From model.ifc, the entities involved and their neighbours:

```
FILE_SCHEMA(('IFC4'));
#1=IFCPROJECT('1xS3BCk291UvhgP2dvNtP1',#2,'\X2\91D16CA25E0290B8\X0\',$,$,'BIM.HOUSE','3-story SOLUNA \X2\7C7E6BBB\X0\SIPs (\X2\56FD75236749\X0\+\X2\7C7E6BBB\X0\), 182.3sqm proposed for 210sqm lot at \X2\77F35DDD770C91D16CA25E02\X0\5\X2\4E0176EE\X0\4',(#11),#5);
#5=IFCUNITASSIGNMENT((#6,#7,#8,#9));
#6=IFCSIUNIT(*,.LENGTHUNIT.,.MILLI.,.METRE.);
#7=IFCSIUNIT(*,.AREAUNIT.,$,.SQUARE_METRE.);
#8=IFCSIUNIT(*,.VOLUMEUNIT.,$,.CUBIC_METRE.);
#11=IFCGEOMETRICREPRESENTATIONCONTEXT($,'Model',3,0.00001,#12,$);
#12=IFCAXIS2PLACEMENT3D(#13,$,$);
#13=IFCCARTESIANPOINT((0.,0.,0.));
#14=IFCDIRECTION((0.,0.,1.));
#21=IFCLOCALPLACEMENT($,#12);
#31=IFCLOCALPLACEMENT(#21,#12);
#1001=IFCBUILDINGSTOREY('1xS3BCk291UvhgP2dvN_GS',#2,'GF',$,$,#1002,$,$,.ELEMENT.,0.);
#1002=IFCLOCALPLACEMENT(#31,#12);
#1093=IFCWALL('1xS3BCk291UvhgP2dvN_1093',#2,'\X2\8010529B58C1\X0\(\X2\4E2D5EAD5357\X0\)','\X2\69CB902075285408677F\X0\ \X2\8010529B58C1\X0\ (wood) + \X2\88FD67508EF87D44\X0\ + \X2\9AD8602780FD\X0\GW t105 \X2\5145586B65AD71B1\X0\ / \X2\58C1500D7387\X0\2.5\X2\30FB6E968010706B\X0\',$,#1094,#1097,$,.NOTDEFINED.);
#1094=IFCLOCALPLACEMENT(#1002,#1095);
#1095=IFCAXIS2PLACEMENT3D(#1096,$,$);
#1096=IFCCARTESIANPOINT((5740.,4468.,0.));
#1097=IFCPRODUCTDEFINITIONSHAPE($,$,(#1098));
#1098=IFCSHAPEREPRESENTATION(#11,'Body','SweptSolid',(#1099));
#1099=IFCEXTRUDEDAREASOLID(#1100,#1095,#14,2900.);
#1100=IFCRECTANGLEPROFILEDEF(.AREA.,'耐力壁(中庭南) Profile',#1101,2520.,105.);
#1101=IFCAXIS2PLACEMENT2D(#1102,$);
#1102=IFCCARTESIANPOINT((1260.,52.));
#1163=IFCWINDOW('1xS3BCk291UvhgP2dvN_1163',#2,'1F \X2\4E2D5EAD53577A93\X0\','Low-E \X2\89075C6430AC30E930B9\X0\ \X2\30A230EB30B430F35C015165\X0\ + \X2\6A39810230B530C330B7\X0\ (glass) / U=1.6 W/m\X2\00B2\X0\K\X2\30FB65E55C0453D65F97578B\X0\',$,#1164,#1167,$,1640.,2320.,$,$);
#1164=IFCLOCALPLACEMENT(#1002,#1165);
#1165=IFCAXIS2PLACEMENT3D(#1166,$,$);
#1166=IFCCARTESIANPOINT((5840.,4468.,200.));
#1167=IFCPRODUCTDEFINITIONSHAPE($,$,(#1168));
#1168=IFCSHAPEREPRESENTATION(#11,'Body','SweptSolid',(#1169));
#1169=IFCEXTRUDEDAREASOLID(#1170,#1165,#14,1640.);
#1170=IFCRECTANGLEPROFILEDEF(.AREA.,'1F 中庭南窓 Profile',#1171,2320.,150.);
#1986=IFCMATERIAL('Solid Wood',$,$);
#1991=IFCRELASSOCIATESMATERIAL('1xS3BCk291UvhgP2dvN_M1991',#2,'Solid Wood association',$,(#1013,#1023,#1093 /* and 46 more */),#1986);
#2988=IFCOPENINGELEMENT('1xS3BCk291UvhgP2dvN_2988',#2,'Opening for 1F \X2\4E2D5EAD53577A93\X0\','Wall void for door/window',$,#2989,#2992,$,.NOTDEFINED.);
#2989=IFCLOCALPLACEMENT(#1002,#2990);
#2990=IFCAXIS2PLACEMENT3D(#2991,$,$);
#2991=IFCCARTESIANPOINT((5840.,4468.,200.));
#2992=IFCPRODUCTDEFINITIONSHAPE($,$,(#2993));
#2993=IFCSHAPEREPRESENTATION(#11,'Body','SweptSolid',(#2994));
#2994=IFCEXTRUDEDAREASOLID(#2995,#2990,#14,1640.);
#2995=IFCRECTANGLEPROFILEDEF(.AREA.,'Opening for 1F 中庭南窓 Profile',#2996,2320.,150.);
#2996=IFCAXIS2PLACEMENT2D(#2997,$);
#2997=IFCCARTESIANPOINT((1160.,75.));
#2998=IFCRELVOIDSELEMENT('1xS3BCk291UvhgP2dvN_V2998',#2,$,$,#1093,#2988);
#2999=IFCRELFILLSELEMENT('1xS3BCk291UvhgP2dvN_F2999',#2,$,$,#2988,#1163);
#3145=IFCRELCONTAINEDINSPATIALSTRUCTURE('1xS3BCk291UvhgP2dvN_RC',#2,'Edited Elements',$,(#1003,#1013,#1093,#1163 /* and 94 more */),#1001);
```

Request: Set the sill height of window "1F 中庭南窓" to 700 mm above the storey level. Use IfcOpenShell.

```python
import numpy as np
import ifcopenshell
import ifcopenshell.api.geometry
import ifcopenshell.geom
import ifcopenshell.util.element
import ifcopenshell.util.placement
import ifcopenshell.util.shape
import ifcopenshell.util.unit

model = ifcopenshell.open("model.ifc")
unit_scale = ifcopenshell.util.unit.calculate_unit_scale(model)

window = model.by_guid("1xS3BCk291UvhgP2dvN_1163")
opening = window.FillsVoids[0].RelatingOpeningElement
storey = ifcopenshell.util.element.get_container(window, ifc_class="IfcBuildingStorey")
level = ifcopenshell.util.placement.get_local_placement(storey.ObjectPlacement)[2, 3]

# The opening's origin need not be at the sill, so measure its lowest point.
shape = ifcopenshell.geom.create_shape(ifcopenshell.geom.settings(), opening)
bottom = ifcopenshell.util.shape.get_shape_bottom_elevation(shape, shape.geometry) / unit_scale
dz = level + 0.7 / unit_scale - bottom

shift = np.array([0.0, 0.0, dz])
# The window is not placed relative to its opening, so move both.
for product in (opening, window):
    matrix = ifcopenshell.util.placement.get_local_placement(product.ObjectPlacement)
    matrix[:3, 3] += shift
    ifcopenshell.api.geometry.edit_object_placement(model, product=product, matrix=matrix, is_si=False)

print(f"moved by {dz * unit_scale:+.3f} m")

model.write("model_rev.ifc")
```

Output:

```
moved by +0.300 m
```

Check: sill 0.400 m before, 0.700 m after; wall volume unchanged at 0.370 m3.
